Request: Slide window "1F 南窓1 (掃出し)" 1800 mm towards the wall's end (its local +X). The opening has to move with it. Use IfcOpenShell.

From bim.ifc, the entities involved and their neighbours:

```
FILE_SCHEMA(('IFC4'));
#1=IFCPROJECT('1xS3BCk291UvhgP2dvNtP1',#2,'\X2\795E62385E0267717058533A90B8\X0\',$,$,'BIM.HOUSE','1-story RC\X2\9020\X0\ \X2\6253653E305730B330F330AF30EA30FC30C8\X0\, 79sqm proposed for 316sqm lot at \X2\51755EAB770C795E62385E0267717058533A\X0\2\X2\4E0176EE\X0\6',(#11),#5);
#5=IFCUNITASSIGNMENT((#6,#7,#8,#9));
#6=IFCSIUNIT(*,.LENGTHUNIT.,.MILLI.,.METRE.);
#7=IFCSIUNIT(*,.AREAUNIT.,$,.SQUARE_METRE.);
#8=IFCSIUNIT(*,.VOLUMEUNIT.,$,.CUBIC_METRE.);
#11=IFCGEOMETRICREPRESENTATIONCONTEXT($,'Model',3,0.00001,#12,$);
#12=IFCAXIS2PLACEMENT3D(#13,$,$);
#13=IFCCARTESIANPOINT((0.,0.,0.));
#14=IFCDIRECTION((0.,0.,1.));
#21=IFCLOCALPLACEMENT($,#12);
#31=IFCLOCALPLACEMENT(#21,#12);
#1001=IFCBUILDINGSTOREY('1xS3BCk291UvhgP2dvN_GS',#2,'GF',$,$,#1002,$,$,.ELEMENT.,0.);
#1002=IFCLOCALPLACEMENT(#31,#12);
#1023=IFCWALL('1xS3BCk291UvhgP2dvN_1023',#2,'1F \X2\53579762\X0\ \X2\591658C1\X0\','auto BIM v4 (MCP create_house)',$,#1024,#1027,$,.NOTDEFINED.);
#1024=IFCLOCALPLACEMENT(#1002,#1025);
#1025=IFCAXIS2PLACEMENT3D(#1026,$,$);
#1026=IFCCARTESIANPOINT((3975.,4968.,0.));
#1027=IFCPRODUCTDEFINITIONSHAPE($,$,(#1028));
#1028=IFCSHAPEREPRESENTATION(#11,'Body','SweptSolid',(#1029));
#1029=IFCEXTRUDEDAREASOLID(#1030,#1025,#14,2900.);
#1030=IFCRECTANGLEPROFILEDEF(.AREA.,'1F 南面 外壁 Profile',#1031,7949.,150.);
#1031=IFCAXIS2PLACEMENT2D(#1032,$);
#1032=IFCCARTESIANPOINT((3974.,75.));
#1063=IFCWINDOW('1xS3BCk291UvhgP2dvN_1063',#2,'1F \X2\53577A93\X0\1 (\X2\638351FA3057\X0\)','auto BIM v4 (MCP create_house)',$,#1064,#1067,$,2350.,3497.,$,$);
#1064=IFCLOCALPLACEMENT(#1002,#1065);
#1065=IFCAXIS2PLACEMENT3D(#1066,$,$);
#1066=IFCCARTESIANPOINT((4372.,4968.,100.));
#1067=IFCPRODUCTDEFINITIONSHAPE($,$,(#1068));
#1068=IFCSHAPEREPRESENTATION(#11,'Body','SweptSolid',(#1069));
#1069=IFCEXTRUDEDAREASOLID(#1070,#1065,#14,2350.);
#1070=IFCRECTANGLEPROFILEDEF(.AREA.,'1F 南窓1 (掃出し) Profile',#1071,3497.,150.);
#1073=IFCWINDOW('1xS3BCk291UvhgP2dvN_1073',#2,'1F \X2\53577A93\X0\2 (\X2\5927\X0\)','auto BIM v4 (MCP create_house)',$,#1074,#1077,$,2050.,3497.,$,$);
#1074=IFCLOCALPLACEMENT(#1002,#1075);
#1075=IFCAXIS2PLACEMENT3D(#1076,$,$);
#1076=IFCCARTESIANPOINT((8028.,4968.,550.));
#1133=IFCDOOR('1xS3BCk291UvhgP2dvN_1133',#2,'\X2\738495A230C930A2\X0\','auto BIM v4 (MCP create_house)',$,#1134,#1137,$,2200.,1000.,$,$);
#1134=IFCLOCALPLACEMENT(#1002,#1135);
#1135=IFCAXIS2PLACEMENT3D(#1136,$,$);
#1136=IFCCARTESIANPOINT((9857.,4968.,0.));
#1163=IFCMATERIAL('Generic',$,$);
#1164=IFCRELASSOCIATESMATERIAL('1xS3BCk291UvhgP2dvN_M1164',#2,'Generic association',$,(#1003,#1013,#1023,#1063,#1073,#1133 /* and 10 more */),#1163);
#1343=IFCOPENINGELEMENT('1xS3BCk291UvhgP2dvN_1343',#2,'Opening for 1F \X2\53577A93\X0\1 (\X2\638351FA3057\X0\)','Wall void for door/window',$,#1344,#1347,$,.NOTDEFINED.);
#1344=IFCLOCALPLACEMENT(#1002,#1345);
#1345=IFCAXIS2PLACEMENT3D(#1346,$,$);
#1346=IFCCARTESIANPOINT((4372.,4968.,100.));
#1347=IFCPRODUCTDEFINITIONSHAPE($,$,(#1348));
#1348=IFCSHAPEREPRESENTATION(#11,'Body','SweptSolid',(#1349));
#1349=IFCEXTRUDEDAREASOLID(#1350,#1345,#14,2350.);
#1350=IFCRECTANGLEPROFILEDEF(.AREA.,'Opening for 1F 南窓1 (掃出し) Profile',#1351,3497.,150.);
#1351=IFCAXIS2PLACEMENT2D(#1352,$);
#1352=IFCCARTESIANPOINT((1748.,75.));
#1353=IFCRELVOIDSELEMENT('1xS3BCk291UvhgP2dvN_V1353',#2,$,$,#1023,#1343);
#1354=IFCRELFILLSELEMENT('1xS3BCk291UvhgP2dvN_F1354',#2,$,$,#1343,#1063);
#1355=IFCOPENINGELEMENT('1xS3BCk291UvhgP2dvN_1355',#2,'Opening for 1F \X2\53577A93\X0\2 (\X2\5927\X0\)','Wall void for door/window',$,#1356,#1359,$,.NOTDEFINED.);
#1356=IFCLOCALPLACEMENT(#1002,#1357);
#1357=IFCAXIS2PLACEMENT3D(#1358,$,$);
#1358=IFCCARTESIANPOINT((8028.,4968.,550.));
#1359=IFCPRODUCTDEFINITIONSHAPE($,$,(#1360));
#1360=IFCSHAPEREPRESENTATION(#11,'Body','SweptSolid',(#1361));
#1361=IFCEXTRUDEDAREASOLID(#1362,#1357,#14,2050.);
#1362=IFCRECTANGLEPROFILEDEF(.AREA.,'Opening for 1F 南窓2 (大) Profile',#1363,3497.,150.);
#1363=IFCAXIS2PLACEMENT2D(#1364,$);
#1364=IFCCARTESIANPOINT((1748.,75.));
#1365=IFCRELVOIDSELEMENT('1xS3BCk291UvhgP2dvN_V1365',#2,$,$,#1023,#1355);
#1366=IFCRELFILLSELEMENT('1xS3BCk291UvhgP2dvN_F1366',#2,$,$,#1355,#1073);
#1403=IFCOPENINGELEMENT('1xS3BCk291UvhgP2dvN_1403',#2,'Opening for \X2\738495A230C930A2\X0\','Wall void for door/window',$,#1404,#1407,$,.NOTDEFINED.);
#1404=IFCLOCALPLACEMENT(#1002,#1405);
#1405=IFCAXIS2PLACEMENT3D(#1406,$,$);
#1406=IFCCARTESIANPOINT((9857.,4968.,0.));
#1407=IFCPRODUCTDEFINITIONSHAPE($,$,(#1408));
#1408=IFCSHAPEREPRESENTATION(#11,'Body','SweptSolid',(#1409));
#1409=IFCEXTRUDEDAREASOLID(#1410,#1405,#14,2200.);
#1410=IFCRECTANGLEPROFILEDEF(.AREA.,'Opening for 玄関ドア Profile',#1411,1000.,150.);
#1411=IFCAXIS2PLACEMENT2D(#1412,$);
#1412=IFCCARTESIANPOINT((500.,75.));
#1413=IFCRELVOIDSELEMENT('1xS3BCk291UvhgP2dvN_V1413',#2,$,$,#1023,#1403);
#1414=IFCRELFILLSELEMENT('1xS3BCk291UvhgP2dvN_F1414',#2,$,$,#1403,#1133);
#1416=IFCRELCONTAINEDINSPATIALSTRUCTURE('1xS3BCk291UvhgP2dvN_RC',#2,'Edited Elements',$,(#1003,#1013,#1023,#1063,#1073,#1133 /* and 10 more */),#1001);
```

```python
import ifcopenshell
import ifcopenshell.api.geometry
import ifcopenshell.util.placement
import ifcopenshell.util.unit

model = ifcopenshell.open("bim.ifc")
unit_scale = ifcopenshell.util.unit.calculate_unit_scale(model)

window = model.by_id(1063)
opening = window.FillsVoids[0].RelatingOpeningElement
wall = opening.VoidsElements[0].RelatingBuildingElement

wall_matrix = ifcopenshell.util.placement.get_local_placement(wall.ObjectPlacement)
shift = wall_matrix[:3, 0] * 1.8 / unit_scale
before = ifcopenshell.util.placement.get_local_placement(window.ObjectPlacement)[:3, 3].copy()

# The window is not placed relative to its opening, so move both.
for product in (opening, window):
    matrix = ifcopenshell.util.placement.get_local_placement(product.ObjectPlacement)
    matrix[:3, 3] += shift
    ifcopenshell.api.geometry.edit_object_placement(model, product=product, matrix=matrix, is_si=False)

after = ifcopenshell.util.placement.get_local_placement(window.ObjectPlacement)[:3, 3]
print("window moved by", (after - before).round(3) + 0.0)

model.write("bim_rev.ifc")
```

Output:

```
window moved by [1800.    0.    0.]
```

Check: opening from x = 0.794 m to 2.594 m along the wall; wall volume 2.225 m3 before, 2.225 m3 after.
